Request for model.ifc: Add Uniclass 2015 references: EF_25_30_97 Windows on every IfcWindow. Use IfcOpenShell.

First a look at what the model holds.

```python
import ifcopenshell

model = ifcopenshell.open("model.ifc")
print(model.schema)
print("classifications:", [c.Name for c in model.by_type("IfcClassification")])
for ifc_class in ("IfcDoor", "IfcRoof", "IfcStair", "IfcWall", "IfcWindow"):
    print(ifc_class, len(model.by_type(ifc_class)))
```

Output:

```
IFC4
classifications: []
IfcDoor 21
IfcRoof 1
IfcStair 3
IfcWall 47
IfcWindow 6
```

```python
import ifcopenshell
import ifcopenshell.api.classification

model = ifcopenshell.open("model.ifc")

system = ifcopenshell.api.classification.add_classification(model, classification="Uniclass 2015")

codes = {
    "IfcWindow": ("EF_25_30_97", "Windows"),
}
for ifc_class, (code, name) in codes.items():
    products = model.by_type(ifc_class)
    ifcopenshell.api.classification.add_reference(
        model, products=products, classification=system, identification=code, name=name
    )
    print(code, len(products))

model.write("model_updated.ifc")
```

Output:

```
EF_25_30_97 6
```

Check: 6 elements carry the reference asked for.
